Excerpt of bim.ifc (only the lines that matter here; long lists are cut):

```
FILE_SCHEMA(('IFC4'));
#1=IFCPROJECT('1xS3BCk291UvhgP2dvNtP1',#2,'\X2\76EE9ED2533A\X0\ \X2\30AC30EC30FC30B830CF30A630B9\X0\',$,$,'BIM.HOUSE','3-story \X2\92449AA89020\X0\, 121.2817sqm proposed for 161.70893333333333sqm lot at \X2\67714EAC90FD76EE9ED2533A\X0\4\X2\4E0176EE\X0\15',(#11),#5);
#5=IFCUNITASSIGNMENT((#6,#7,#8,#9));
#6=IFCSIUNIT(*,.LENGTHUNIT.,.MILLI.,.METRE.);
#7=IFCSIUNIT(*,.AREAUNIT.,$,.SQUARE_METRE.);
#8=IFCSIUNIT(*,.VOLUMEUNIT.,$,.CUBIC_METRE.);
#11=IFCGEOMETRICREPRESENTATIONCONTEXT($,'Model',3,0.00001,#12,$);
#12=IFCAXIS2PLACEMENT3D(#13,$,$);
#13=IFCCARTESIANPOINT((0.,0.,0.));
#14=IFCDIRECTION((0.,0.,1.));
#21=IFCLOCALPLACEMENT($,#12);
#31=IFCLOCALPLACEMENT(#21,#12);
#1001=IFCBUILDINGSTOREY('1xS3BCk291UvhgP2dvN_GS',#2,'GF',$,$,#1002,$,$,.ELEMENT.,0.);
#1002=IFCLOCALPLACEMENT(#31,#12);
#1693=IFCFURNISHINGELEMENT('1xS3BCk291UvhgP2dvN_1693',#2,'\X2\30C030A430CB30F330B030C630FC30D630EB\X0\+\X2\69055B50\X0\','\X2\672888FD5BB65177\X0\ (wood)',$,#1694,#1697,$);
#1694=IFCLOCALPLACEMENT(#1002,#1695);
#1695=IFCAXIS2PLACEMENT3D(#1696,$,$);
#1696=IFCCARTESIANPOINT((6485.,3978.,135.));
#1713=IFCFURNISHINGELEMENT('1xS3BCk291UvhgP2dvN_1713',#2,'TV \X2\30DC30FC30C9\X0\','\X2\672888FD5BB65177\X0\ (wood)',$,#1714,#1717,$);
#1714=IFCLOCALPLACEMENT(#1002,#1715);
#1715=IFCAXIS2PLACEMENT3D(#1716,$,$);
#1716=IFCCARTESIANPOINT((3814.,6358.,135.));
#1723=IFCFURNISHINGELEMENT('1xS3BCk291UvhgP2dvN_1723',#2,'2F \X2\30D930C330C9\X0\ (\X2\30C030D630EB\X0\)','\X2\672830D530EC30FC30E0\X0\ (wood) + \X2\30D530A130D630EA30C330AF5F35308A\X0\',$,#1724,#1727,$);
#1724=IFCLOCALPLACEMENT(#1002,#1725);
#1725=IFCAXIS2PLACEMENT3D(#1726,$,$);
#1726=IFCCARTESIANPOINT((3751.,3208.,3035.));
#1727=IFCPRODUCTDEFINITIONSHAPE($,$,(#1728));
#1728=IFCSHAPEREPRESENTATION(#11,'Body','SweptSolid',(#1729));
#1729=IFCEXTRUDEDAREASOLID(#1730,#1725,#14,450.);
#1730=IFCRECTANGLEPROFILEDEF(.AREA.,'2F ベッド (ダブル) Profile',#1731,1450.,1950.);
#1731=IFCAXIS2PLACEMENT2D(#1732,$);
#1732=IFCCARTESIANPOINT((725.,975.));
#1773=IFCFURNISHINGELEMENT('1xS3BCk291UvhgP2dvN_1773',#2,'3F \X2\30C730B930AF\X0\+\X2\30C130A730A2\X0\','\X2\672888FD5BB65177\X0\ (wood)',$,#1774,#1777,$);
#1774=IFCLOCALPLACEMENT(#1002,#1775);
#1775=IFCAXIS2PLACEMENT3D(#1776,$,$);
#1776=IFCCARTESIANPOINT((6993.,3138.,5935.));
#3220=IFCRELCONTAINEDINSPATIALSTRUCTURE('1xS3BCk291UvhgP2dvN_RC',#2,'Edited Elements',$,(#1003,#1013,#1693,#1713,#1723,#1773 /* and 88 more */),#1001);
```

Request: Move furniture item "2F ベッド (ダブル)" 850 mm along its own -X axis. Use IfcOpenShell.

```python
import ifcopenshell
import ifcopenshell.api.geometry
import ifcopenshell.util.placement

model = ifcopenshell.open("bim.ifc")

item = model.by_guid("1xS3BCk291UvhgP2dvN_1723")
matrix = ifcopenshell.util.placement.get_local_placement(item.ObjectPlacement)
matrix[:3, 3] -= matrix[:3, 0] * 850.0
ifcopenshell.api.geometry.edit_object_placement(model, product=item, matrix=matrix, is_si=False)

print(ifcopenshell.util.placement.get_local_placement(item.ObjectPlacement).round(3) + 0.0)

model.write("bim_rev.ifc")
```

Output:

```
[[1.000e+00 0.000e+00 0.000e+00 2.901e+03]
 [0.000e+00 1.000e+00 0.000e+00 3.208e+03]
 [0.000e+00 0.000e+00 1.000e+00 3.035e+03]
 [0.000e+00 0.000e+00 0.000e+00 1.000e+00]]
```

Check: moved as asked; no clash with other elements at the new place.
